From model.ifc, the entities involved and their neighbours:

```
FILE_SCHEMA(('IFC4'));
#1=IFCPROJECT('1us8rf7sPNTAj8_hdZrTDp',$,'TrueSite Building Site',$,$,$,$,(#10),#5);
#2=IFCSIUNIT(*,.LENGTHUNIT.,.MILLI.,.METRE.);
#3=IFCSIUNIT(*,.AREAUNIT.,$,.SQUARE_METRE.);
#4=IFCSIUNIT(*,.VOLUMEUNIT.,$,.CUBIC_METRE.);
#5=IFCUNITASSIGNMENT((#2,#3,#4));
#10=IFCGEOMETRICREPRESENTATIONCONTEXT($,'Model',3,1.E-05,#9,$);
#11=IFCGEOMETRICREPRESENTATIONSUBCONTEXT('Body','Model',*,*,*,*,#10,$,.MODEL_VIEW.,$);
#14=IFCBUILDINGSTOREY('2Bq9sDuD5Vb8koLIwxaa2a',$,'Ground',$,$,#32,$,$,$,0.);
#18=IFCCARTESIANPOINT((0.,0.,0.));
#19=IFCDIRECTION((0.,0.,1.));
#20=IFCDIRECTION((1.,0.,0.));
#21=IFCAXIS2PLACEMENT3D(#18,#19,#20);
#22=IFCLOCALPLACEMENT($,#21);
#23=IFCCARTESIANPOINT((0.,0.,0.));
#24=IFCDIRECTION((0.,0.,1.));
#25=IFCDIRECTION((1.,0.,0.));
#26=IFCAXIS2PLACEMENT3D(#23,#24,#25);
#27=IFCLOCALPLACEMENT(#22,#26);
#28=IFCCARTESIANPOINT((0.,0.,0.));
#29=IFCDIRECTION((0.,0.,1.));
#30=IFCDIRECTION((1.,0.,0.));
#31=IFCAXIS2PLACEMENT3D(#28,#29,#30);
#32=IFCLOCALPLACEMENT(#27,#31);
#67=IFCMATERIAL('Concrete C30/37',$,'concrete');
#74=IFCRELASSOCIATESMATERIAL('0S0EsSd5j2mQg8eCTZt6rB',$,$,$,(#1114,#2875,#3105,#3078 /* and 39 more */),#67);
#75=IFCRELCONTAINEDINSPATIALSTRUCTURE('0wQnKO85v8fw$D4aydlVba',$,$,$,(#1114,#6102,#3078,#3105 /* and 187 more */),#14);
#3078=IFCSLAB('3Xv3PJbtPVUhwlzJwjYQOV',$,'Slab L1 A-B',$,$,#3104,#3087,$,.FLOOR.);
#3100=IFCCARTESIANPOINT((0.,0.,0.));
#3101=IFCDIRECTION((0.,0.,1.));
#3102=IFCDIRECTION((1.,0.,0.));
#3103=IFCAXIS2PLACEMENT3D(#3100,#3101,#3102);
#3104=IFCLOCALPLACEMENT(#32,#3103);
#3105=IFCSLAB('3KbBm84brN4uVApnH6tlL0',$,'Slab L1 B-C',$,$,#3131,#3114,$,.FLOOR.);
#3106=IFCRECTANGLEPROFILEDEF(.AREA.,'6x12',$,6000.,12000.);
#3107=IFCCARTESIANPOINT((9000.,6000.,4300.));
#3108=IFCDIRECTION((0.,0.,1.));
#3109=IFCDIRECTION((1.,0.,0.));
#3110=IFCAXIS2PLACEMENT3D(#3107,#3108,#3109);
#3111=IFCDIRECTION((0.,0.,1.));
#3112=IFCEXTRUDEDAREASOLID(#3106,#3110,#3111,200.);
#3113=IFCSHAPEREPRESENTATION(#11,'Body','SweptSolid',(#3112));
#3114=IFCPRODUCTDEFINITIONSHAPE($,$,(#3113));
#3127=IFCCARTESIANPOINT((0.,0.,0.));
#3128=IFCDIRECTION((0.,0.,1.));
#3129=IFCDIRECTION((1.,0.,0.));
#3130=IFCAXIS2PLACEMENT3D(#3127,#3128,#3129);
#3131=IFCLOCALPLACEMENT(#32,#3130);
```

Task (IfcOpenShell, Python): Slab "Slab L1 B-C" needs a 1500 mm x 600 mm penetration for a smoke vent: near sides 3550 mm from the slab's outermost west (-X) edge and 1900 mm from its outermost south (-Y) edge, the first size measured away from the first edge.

```python
import numpy as np
import ifcopenshell
import ifcopenshell.api.feature
import ifcopenshell.api.geometry
import ifcopenshell.api.root
import ifcopenshell.geom
import ifcopenshell.util.placement
import ifcopenshell.util.representation
import ifcopenshell.util.shape
import ifcopenshell.util.unit

model = ifcopenshell.open("model.ifc")
unit_scale = ifcopenshell.util.unit.calculate_unit_scale(model)
settings = ifcopenshell.geom.settings()


def volume(element):
    """Net volume in cubic metres, openings subtracted."""
    shape = ifcopenshell.geom.create_shape(settings, element)
    return ifcopenshell.util.shape.get_volume(shape.geometry)


slab = model.by_id(3105)
before = volume(slab)

# Extent in the slab's own axes, in metres. The edges named are its -X and -Y sides.
slab_shape = ifcopenshell.geom.create_shape(settings, slab)
vertices = ifcopenshell.util.shape.get_vertices(slab_shape.geometry)
x_min, y_min, bottom = vertices.min(axis=0)
top = vertices[:, 2].max()

opening = ifcopenshell.api.root.create_entity(model, ifc_class="IfcOpeningElement", name="Smoke vent opening", predefined_type="OPENING")
context = ifcopenshell.util.representation.get_context(model, "Model", "Body", "MODEL_VIEW")
width, depth = 1.5, 0.6
outline = [(0.0, 0.0), (width, 0.0), (width, depth), (0.0, depth), (0.0, 0.0)]
# Overshoot both faces by 50 mm so the cut is clean.
shape = ifcopenshell.api.geometry.add_slab_representation(
    model, context=context, depth=top - bottom + 0.1, polyline=outline
)
ifcopenshell.api.geometry.assign_representation(model, product=opening, representation=shape)

matrix = ifcopenshell.util.placement.get_local_placement(slab.ObjectPlacement)
matrix[:, 3] = matrix @ np.append(np.array([x_min + 3.55, y_min + 1.9, bottom - 0.05]) / unit_scale, 1.0)
ifcopenshell.api.geometry.edit_object_placement(model, product=opening, matrix=matrix, is_si=False)
ifcopenshell.api.feature.add_feature(model, feature=opening, element=slab)

after = volume(slab)

print(f"slab volume {before:.3f} -> {after:.3f} m3")

model.write("model_updated.ifc")
```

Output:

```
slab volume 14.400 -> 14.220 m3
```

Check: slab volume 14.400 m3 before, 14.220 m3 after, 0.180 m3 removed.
